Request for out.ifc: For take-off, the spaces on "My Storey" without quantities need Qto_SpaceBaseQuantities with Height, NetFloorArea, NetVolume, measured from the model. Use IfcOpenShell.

First a look at what the model holds.

```python
import ifcopenshell
import ifcopenshell.util.element
import ifcopenshell.util.unit

model = ifcopenshell.open("out.ifc")
print(model.schema)
for unit_type in ("LENGTHUNIT", "AREAUNIT", "VOLUMEUNIT"):
    print(unit_type, ifcopenshell.util.unit.calculate_unit_scale(model, unit_type))
storey = next(s for s in model.by_type("IfcBuildingStorey") if s.Name == "My Storey")
spaces = [e for e in ifcopenshell.util.element.get_decomposition(storey) if e.is_a("IfcSpace")]
for e in sorted(spaces, key=lambda e: e.id()):
    print(e.id(), e.is_a(), e.Name, list(ifcopenshell.util.element.get_psets(e, qtos_only=True)), sep=" | ")
```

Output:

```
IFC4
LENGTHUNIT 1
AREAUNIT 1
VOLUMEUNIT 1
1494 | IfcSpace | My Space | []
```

```python
import ifcopenshell
import ifcopenshell.api.pset
import ifcopenshell.geom
import ifcopenshell.util.element
import ifcopenshell.util.shape
import ifcopenshell.util.unit

model = ifcopenshell.open("out.ifc")
unit_scale = ifcopenshell.util.unit.calculate_unit_scale(model)
area_scale = ifcopenshell.util.unit.calculate_unit_scale(model, "AREAUNIT")
volume_scale = ifcopenshell.util.unit.calculate_unit_scale(model, "VOLUMEUNIT")
settings = ifcopenshell.geom.settings()

storey = next(s for s in model.by_type("IfcBuildingStorey") if s.Name == "My Storey")
spaces = [e for e in ifcopenshell.util.element.get_decomposition(storey) if e.is_a("IfcSpace")]

for e in sorted(spaces, key=lambda e: e.id()):
    if ifcopenshell.util.element.get_psets(e, qtos_only=True, should_inherit=False):
        continue
    # Geometry comes back in metres, in the element's own axes.
    shape = ifcopenshell.geom.create_shape(settings, e)
    values = {
        "Height": ifcopenshell.util.shape.get_z(shape.geometry) / unit_scale,
        "NetFloorArea": ifcopenshell.util.shape.get_footprint_area(shape.geometry) / area_scale,
        "NetVolume": ifcopenshell.util.shape.get_volume(shape.geometry) / volume_scale,
    }
    qto = ifcopenshell.api.pset.add_qto(model, product=e, name="Qto_SpaceBaseQuantities")
    ifcopenshell.api.pset.edit_qto(model, qto=qto, properties=values)
    print(e.id(), {k: round(v, 3) for k, v in values.items()})

model.write("out_v2.ifc")
```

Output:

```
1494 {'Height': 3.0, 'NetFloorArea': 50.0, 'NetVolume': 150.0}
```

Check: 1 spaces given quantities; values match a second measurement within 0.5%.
